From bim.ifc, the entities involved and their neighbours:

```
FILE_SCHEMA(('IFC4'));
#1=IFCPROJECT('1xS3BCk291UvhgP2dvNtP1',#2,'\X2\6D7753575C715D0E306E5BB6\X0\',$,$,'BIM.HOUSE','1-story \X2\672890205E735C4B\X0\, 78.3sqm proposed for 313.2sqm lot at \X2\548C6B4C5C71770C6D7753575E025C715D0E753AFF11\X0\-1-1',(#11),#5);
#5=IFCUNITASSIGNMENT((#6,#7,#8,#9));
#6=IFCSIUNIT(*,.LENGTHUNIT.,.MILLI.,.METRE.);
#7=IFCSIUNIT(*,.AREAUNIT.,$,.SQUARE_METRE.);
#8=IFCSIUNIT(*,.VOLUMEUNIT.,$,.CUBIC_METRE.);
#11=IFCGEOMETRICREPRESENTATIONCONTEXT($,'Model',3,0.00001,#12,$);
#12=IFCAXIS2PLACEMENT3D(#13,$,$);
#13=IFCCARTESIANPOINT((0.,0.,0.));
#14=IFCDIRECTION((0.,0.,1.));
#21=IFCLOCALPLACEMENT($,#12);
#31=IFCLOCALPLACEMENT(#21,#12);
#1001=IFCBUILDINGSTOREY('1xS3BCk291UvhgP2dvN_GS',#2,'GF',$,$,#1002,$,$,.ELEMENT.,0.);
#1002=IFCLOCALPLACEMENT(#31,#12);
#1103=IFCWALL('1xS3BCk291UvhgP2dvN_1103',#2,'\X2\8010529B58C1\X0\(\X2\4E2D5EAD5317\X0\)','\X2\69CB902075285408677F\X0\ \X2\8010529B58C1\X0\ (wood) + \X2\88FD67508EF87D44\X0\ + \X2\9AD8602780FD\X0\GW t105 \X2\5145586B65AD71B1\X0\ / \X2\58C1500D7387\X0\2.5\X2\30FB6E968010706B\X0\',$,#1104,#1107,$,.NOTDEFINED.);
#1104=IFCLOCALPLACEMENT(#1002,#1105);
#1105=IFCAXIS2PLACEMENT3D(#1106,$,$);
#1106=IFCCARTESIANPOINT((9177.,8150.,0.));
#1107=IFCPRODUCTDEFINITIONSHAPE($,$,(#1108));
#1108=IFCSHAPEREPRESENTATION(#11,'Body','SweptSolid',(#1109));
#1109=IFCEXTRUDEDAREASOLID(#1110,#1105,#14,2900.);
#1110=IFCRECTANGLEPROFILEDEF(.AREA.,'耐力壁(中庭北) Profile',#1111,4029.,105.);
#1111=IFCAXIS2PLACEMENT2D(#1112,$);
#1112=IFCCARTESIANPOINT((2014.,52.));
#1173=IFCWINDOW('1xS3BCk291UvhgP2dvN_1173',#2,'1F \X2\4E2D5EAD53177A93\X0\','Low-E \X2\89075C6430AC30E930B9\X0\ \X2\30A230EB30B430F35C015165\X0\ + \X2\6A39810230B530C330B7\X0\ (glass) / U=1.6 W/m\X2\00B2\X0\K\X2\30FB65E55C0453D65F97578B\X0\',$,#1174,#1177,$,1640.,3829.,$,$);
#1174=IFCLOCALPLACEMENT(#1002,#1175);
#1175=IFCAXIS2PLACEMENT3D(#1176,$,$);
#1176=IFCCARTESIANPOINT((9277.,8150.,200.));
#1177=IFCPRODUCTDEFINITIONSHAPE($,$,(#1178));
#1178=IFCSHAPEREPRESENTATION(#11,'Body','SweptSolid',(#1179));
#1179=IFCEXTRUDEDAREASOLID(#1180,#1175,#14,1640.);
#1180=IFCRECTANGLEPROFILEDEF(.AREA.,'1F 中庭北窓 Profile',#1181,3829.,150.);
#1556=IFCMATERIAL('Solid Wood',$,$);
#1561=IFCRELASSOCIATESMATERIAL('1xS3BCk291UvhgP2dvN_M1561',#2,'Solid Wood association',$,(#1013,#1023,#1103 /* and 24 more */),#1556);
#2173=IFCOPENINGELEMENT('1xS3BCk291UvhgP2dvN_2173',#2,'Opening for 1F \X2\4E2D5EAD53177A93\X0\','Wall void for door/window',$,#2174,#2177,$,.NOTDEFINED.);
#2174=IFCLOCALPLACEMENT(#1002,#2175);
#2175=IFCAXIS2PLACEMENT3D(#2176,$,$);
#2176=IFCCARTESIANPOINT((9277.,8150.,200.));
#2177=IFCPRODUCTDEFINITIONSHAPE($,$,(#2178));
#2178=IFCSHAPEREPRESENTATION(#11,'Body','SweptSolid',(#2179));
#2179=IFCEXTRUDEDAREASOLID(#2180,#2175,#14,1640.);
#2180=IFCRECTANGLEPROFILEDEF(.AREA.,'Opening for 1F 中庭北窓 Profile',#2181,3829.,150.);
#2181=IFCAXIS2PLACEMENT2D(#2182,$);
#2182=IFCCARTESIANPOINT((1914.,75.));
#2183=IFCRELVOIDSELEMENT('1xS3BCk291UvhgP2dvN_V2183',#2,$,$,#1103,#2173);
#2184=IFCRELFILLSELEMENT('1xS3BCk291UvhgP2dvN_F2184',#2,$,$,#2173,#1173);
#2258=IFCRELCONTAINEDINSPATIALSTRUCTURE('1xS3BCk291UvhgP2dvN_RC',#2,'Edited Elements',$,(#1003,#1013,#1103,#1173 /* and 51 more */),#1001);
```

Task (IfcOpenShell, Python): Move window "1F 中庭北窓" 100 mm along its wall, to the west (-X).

```python
import ifcopenshell
import ifcopenshell.api.geometry
import ifcopenshell.util.placement
import ifcopenshell.util.unit

model = ifcopenshell.open("bim.ifc")
unit_scale = ifcopenshell.util.unit.calculate_unit_scale(model)

window = model.by_guid("1xS3BCk291UvhgP2dvN_1173")
opening = window.FillsVoids[0].RelatingOpeningElement
wall = opening.VoidsElements[0].RelatingBuildingElement

wall_matrix = ifcopenshell.util.placement.get_local_placement(wall.ObjectPlacement)
shift = wall_matrix[:3, 0] * -0.1 / unit_scale
before = ifcopenshell.util.placement.get_local_placement(window.ObjectPlacement)[:3, 3].copy()

# The window is not placed relative to its opening, so move both.
for product in (opening, window):
    matrix = ifcopenshell.util.placement.get_local_placement(product.ObjectPlacement)
    matrix[:3, 3] += shift
    ifcopenshell.api.geometry.edit_object_placement(model, product=product, matrix=matrix, is_si=False)

after = ifcopenshell.util.placement.get_local_placement(window.ObjectPlacement)[:3, 3]
print("window moved by", (after - before).round(3) + 0.0)

model.write("bim_rev.ifc")
```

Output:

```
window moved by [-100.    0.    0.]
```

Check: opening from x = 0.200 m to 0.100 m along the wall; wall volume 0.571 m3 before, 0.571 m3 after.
